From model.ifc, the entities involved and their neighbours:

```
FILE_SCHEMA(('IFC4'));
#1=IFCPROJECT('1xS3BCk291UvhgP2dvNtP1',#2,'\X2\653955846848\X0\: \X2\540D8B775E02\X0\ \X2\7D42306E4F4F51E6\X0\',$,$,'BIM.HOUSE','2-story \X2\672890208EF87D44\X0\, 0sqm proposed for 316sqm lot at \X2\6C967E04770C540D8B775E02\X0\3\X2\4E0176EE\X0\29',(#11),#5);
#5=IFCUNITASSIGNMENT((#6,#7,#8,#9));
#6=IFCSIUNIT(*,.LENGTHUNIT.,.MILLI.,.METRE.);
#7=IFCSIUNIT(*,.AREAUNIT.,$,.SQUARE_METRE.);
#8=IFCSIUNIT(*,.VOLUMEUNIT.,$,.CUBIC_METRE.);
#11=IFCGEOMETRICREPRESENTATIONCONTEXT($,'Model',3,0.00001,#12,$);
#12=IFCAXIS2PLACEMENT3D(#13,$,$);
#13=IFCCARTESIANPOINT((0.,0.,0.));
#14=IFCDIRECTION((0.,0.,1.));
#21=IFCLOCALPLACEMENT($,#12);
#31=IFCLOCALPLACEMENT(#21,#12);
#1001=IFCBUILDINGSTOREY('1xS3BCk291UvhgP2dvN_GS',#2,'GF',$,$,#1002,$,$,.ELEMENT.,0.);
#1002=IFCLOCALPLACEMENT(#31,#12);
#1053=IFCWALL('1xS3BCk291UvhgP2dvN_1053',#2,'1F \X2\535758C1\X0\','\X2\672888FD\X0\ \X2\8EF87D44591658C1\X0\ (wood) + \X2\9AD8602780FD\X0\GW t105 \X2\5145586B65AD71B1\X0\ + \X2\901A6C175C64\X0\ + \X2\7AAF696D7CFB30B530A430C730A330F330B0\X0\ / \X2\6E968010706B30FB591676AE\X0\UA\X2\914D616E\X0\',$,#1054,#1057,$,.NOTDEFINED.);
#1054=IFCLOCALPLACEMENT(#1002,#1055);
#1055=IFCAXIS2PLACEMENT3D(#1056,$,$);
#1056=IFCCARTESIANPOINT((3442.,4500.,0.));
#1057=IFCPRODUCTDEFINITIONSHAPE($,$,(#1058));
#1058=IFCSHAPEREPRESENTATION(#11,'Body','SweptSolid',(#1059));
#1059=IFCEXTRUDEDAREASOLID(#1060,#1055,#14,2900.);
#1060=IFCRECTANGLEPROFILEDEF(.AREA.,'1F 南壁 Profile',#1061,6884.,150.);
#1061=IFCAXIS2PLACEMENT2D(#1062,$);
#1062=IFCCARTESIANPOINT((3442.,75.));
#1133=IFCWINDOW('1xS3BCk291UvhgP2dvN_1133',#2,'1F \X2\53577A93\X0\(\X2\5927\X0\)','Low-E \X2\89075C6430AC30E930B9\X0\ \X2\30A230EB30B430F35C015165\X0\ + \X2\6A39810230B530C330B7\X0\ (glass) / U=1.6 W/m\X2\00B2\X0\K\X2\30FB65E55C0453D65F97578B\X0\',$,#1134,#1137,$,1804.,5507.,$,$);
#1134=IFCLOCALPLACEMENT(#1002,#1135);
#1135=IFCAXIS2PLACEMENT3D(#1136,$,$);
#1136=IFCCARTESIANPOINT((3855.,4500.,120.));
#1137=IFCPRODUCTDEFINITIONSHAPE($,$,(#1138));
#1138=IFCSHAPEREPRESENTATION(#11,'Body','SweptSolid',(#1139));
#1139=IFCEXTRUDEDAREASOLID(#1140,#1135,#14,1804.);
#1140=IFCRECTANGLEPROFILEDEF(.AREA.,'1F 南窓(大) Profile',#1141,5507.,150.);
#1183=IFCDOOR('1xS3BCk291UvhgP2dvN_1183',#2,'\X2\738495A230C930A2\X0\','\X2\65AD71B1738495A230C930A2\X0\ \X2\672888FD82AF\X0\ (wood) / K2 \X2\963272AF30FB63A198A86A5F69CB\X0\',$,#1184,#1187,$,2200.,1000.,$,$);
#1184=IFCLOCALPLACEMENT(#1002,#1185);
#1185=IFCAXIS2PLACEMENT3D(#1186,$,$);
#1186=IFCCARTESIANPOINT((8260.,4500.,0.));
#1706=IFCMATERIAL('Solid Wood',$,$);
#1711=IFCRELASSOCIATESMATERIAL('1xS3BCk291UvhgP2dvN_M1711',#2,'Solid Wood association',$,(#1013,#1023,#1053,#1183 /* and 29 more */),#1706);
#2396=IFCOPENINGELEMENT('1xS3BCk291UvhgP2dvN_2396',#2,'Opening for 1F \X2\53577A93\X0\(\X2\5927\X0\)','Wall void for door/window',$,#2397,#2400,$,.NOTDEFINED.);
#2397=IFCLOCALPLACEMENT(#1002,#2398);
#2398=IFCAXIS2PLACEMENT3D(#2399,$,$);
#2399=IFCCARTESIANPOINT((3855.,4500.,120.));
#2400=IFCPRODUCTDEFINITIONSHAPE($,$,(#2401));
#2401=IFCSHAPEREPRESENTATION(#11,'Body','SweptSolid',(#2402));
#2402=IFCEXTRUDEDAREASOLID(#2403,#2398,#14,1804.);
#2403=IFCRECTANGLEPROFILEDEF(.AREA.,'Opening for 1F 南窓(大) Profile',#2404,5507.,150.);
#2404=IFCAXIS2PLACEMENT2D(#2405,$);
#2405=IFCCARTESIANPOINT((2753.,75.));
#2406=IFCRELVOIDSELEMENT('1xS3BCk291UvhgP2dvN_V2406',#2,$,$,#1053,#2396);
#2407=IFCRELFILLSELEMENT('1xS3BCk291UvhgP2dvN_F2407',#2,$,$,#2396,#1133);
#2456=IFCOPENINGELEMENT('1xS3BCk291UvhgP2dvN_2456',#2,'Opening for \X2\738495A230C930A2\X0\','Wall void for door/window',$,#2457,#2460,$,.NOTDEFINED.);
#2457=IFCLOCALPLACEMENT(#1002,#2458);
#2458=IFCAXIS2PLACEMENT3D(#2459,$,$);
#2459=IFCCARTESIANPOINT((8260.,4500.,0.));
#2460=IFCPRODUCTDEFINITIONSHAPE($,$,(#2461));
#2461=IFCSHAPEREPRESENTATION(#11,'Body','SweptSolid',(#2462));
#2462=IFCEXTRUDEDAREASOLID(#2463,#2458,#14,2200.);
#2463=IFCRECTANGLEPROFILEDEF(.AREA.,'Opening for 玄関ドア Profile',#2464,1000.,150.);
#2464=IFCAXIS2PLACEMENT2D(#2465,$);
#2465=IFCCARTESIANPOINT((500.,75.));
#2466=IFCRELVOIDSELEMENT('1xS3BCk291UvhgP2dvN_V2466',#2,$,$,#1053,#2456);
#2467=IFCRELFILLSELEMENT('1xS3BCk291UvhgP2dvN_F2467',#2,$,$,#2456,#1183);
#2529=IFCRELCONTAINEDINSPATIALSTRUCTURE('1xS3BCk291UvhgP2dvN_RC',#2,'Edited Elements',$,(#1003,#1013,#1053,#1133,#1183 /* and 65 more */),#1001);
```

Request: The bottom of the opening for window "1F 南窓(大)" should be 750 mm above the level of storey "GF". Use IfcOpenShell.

```python
import numpy as np
import ifcopenshell
import ifcopenshell.api.geometry
import ifcopenshell.geom
import ifcopenshell.util.element
import ifcopenshell.util.placement
import ifcopenshell.util.shape
import ifcopenshell.util.unit

model = ifcopenshell.open("model.ifc")
unit_scale = ifcopenshell.util.unit.calculate_unit_scale(model)

window = model.by_guid("1xS3BCk291UvhgP2dvN_1133")
opening = window.FillsVoids[0].RelatingOpeningElement
storey = ifcopenshell.util.element.get_container(window, ifc_class="IfcBuildingStorey")
level = ifcopenshell.util.placement.get_local_placement(storey.ObjectPlacement)[2, 3]

# The opening's origin need not be at the sill, so measure its lowest point.
shape = ifcopenshell.geom.create_shape(ifcopenshell.geom.settings(), opening)
bottom = ifcopenshell.util.shape.get_shape_bottom_elevation(shape, shape.geometry) / unit_scale
dz = level + 750.0 - bottom

shift = np.array([0.0, 0.0, dz])
# The window is not placed relative to its opening, so move both.
for product in (opening, window):
    matrix = ifcopenshell.util.placement.get_local_placement(product.ObjectPlacement)
    matrix[:3, 3] += shift
    ifcopenshell.api.geometry.edit_object_placement(model, product=product, matrix=matrix, is_si=False)

print(f"moved by {dz * unit_scale:+.3f} m")

model.write("model_rev.ifc")
```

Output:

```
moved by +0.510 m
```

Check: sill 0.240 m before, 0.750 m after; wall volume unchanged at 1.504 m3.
